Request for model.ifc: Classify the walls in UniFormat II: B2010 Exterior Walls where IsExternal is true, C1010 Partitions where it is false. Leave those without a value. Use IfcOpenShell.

First a look at what the model holds.

```python
import ifcopenshell
import ifcopenshell.util.element

model = ifcopenshell.open("model.ifc")
print(model.schema)
print("classifications:", [c.Name for c in model.by_type("IfcClassification")])
values = [ifcopenshell.util.element.get_pset(e, "Pset_WallCommon", "IsExternal") for e in model.by_type("IfcWall")]
for value in (True, False, None):
    print("IsExternal", value, values.count(value))
```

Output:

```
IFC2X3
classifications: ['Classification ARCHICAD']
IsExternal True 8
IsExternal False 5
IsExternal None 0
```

```python
import ifcopenshell
import ifcopenshell.api.classification
import ifcopenshell.util.element

model = ifcopenshell.open("model.ifc")

# IFC2X3 requires Source and Edition and has no link from the project to the system.
system = model.create_entity("IfcClassification", Source="ASTM", Edition="E1557", Name="UniFormat II")

walls = model.by_type("IfcWall")
external = {e: ifcopenshell.util.element.get_pset(e, "Pset_WallCommon", "IsExternal") for e in walls}
for flag, code, name in ((True, "B2010", "Exterior Walls"), (False, "C1010", "Partitions")):
    products = [e for e in walls if external[e] is flag]
    ifcopenshell.api.classification.add_reference(
        model, products=products, classification=system, identification=code, name=name
    )
    print(code, len(products))

model.write("model_edited.ifc")
```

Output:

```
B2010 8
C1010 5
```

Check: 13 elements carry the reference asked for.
